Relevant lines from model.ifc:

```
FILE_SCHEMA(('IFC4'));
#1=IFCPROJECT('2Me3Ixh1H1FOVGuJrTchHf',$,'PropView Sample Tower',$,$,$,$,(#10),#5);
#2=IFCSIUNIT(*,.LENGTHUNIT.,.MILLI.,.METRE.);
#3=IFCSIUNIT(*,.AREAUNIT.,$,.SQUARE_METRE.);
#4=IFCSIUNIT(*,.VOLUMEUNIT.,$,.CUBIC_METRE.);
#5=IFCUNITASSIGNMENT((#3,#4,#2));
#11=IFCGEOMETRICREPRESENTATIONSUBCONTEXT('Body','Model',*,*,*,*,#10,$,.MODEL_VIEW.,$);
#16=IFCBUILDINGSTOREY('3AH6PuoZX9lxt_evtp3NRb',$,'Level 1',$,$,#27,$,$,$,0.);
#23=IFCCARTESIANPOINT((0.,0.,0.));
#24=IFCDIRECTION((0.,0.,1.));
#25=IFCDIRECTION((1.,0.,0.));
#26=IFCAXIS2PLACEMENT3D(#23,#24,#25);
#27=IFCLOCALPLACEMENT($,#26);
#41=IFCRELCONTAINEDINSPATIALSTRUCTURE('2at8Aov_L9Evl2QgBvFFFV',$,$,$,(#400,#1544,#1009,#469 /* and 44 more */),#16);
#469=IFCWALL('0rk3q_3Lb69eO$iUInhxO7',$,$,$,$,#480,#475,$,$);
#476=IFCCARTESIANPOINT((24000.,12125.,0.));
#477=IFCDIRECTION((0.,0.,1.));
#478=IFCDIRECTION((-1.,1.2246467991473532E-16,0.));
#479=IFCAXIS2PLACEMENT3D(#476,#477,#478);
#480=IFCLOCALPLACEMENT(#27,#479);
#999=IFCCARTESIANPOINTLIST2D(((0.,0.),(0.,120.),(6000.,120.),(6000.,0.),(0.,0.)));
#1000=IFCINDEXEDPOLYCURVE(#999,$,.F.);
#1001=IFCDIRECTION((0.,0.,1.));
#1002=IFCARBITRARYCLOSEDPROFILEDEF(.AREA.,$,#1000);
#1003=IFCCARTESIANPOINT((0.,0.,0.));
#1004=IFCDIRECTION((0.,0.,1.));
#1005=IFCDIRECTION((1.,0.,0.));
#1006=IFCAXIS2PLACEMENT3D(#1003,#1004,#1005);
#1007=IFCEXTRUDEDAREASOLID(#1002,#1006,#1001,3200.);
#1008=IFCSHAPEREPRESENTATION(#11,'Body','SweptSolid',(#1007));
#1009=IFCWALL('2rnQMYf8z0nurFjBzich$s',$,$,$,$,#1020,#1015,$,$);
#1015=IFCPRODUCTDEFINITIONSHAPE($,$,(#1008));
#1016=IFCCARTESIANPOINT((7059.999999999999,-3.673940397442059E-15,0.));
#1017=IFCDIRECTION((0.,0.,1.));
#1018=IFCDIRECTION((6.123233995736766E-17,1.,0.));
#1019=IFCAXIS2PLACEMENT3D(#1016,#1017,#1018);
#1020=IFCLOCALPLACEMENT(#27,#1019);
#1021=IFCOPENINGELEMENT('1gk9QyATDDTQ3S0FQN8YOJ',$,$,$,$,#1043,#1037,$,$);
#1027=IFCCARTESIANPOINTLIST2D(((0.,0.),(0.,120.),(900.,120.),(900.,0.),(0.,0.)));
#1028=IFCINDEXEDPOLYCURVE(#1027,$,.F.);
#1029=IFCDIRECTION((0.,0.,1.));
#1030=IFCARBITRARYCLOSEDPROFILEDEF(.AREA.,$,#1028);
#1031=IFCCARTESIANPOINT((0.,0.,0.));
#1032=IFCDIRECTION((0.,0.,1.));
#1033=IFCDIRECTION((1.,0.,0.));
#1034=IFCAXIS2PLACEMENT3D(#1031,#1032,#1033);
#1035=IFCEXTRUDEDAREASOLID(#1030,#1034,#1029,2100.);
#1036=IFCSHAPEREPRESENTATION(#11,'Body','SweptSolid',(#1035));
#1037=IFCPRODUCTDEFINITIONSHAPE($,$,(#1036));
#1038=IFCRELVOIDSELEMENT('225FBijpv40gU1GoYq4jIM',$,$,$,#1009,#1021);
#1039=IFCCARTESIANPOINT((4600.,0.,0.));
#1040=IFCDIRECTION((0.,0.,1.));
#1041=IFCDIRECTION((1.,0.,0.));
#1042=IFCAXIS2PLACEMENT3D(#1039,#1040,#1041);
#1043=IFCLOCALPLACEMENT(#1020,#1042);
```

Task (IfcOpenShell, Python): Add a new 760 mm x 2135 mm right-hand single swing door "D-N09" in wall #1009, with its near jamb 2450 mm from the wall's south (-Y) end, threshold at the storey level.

```python
import numpy as np
import ifcopenshell
import ifcopenshell.api.feature
import ifcopenshell.api.geometry
import ifcopenshell.api.root
import ifcopenshell.api.spatial
import ifcopenshell.geom
import ifcopenshell.util.element
import ifcopenshell.util.placement
import ifcopenshell.util.representation
import ifcopenshell.util.shape
import ifcopenshell.util.unit

model = ifcopenshell.open("model.ifc")
unit_scale = ifcopenshell.util.unit.calculate_unit_scale(model)
settings = ifcopenshell.geom.settings()


def volume(element):
    """Net volume in cubic metres, openings subtracted."""
    shape = ifcopenshell.geom.create_shape(settings, element)
    return ifcopenshell.util.shape.get_volume(shape.geometry)


wall = model.by_guid("2rnQMYf8z0nurFjBzich$s")
storey = ifcopenshell.util.element.get_container(wall, ifc_class="IfcBuildingStorey")
context = ifcopenshell.util.representation.get_context(model, "Model", "Body", "MODEL_VIEW")
before = volume(wall)

width, height, from_end, sill = 0.76, 2.135, 2.45, 0.0  # metres

# The wall runs along its own X axis, and the end named is its -X end.
wall_shape = ifcopenshell.geom.create_shape(settings, wall)
x, y, z = ifcopenshell.util.shape.get_vertices(wall_shape.geometry).T
start = x.min() + from_end
face, thickness = float(y.min()), float(y.max() - y.min())
wall_matrix = ifcopenshell.util.placement.get_local_placement(wall.ObjectPlacement)
level = ifcopenshell.util.placement.get_local_placement(storey.ObjectPlacement)[2, 3]


def in_wall(x, y):
    """Placement at x, y metres in the wall's axes, at sill height."""
    matrix = wall_matrix.copy()
    matrix[:, 3] = wall_matrix @ np.array([x / unit_scale, y / unit_scale, 0.0, 1.0])
    matrix[2, 3] = level + sill / unit_scale
    return matrix


# Opening: a box that overshoots both wall faces by 50 mm.
opening = ifcopenshell.api.root.create_entity(model, ifc_class="IfcOpeningElement", predefined_type="OPENING")
box = ifcopenshell.api.geometry.add_wall_representation(
    model, context=context, length=width, height=height, thickness=thickness + 0.1
)
ifcopenshell.api.geometry.assign_representation(model, product=opening, representation=box)
ifcopenshell.api.geometry.edit_object_placement(model, product=opening, matrix=in_wall(start, face - 0.05), is_si=False)
ifcopenshell.api.feature.add_feature(model, feature=opening, element=wall)

door = ifcopenshell.api.root.create_entity(model, ifc_class="IfcDoor", name="D-N09", predefined_type="DOOR")
door.OverallWidth, door.OverallHeight = width / unit_scale, height / unit_scale
door.OperationType = "SINGLE_SWING_RIGHT"
body = ifcopenshell.api.geometry.add_door_representation(
    model,
    context=context,
    overall_width=door.OverallWidth,
    overall_height=door.OverallHeight,
    operation_type="SINGLE_SWING_RIGHT",
    lining_properties={"LiningDepth": thickness / unit_scale, "ThresholdDepth": thickness / unit_scale},
)
ifcopenshell.api.geometry.assign_representation(model, product=door, representation=body)
ifcopenshell.api.spatial.assign_container(model, products=[door], relating_structure=storey)
ifcopenshell.api.feature.add_filling(model, opening=opening, element=door)

# The lining spans the wall, so the door starts at the wall face.
ifcopenshell.api.geometry.edit_object_placement(model, product=door, matrix=in_wall(start, face), is_si=False)

after = volume(wall)

print(f"wall volume {before:.3f} -> {after:.3f} m3")

model.write("model_v2.ifc")
```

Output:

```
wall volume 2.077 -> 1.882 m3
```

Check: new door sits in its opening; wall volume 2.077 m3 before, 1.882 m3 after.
